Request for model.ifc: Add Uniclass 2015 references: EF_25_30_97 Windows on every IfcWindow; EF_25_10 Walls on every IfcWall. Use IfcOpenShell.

First a look at what the model holds.

```python
import ifcopenshell

model = ifcopenshell.open("model.ifc")
print(model.schema)
print("classifications:", [c.Name for c in model.by_type("IfcClassification")])
for ifc_class in ("IfcDoor", "IfcRoof", "IfcStair", "IfcWall", "IfcWindow"):
    print(ifc_class, len(model.by_type(ifc_class)))
```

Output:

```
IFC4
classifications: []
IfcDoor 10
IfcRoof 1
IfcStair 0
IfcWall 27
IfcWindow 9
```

```python
import ifcopenshell
import ifcopenshell.api.classification

model = ifcopenshell.open("model.ifc")

system = ifcopenshell.api.classification.add_classification(model, classification="Uniclass 2015")

codes = {
    "IfcWindow": ("EF_25_30_97", "Windows"),
    "IfcWall": ("EF_25_10", "Walls"),
}
for ifc_class, (code, name) in codes.items():
    products = model.by_type(ifc_class)
    ifcopenshell.api.classification.add_reference(
        model, products=products, classification=system, identification=code, name=name
    )
    print(code, len(products))

model.write("model_v2.ifc")
```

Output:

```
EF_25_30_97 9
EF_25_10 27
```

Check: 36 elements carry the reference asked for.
